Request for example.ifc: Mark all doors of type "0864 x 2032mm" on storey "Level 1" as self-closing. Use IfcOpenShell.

First a look at what the model holds.

```python
import ifcopenshell
import ifcopenshell.util.element

model = ifcopenshell.open("example.ifc")
print(model.schema)
storey = next(s for s in model.by_type("IfcBuildingStorey") if s.Name == "Level 1")
doors = [e for e in ifcopenshell.util.element.get_decomposition(storey) if e.is_a("IfcDoor")]
seen = {}
for e in doors:
    element_type = ifcopenshell.util.element.get_type(e)
    key = (element_type.Name if element_type != e and element_type else None, ifcopenshell.util.element.get_pset(e, "Pset_DoorCommon", "SelfClosing"))
    seen[key] = seen.get(key, 0) + 1
for (name, value), count in sorted(seen.items(), key=str):
    print(count, "x", name, "|", value)
```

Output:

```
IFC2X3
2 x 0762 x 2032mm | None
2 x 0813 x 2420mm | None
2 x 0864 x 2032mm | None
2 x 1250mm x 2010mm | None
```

```python
import ifcopenshell
import ifcopenshell.api.pset
import ifcopenshell.util.element

model = ifcopenshell.open("example.ifc")

storey = next(s for s in model.by_type("IfcBuildingStorey") if s.Name == "Level 1")
doors = [e for e in ifcopenshell.util.element.get_decomposition(storey) if e.is_a("IfcDoor")]

count = 0
for e in doors:
    element_type = ifcopenshell.util.element.get_type(e)
    if element_type in (None, e) or element_type.Name != "0864 x 2032mm":
        continue
    # add_pset returns the element's existing set when there is one.
    pset = ifcopenshell.api.pset.add_pset(model, product=e, name="Pset_DoorCommon")
    ifcopenshell.api.pset.edit_pset(model, pset=pset, properties={"SelfClosing": True})
    count += 1

print(count, "doors updated")

model.write("example_updated.ifc")
```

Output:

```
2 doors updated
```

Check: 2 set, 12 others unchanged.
